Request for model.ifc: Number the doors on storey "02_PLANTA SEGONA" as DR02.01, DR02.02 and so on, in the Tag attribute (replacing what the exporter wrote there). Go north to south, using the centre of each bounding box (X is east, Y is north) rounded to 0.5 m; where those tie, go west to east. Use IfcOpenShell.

First a look at what the model holds.

```python
import ifcopenshell
import ifcopenshell.util.element
import ifcopenshell.util.placement

model = ifcopenshell.open("model.ifc")
print(model.schema)
storey = next(s for s in model.by_type("IfcBuildingStorey") if s.Name == "02_PLANTA SEGONA")
doors = [e for e in ifcopenshell.util.element.get_decomposition(storey) if e.is_a("IfcDoor")]
for e in sorted(doors, key=lambda e: e.id()):
    origin = ifcopenshell.util.placement.get_local_placement(e.ObjectPlacement)[:3, 3]
    print(e.id(), e.Tag, e.Name, origin.round(2) + 0.0, sep=" | ")
```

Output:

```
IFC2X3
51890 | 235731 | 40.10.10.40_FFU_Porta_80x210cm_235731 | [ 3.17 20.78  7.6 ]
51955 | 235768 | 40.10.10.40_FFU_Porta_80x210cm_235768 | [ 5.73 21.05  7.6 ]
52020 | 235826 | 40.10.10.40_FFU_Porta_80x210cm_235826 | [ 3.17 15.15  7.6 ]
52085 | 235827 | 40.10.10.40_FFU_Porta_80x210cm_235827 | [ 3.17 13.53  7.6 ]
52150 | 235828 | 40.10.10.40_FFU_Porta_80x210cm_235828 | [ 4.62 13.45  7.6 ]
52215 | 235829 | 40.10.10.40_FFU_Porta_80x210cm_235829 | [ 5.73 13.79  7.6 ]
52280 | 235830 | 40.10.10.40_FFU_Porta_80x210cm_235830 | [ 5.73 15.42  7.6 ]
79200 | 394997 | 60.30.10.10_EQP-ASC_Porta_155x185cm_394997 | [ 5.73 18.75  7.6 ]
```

```python
import ifcopenshell
import ifcopenshell.geom
import ifcopenshell.util.element
import ifcopenshell.util.shape

model = ifcopenshell.open("model.ifc")
settings = ifcopenshell.geom.settings()
settings.set("use-world-coords", True)


def centre(element):
    shape = ifcopenshell.geom.create_shape(settings, element)
    return ifcopenshell.util.shape.get_bbox_centroid(shape.geometry)


storey = next(s for s in model.by_type("IfcBuildingStorey") if s.Name == "02_PLANTA SEGONA")
doors = [e for e in ifcopenshell.util.element.get_decomposition(storey) if e.is_a("IfcDoor")]

# Insertion points can sit at a corner or the storey origin, so sort by the geometry (in metres).
centres = {e: centre(e) for e in doors}
doors.sort(key=lambda e: (-round(centres[e][1] / 0.5), centres[e][0]))

for i, e in enumerate(doors, start=1):
    number = f"DR02.{i:02d}"
    e.Tag = number
    print(e.id(), number)

model.write("model_v2.ifc")
```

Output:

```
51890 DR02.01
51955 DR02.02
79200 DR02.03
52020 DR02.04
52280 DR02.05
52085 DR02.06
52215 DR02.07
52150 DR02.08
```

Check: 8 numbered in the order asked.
